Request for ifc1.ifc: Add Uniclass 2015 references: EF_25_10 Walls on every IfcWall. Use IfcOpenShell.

First a look at what the model holds.

```python
import ifcopenshell

model = ifcopenshell.open("ifc1.ifc")
print(model.schema)
print("classifications:", [c.Name for c in model.by_type("IfcClassification")])
for ifc_class in ("IfcDoor", "IfcRoof", "IfcStair", "IfcWall", "IfcWindow"):
    print(ifc_class, len(model.by_type(ifc_class)))
```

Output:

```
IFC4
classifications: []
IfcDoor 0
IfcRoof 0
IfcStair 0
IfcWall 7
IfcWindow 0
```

```python
import ifcopenshell
import ifcopenshell.api.classification

model = ifcopenshell.open("ifc1.ifc")

system = ifcopenshell.api.classification.add_classification(model, classification="Uniclass 2015")

codes = {
    "IfcWall": ("EF_25_10", "Walls"),
}
for ifc_class, (code, name) in codes.items():
    products = model.by_type(ifc_class)
    ifcopenshell.api.classification.add_reference(
        model, products=products, classification=system, identification=code, name=name
    )
    print(code, len(products))

model.write("ifc1_rev.ifc")
```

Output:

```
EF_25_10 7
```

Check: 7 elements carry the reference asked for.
